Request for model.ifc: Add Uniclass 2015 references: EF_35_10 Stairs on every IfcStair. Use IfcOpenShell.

First a look at what the model holds.

```python
import ifcopenshell

model = ifcopenshell.open("model.ifc")
print(model.schema)
print("classifications:", [c.Name for c in model.by_type("IfcClassification")])
for ifc_class in ("IfcDoor", "IfcRoof", "IfcStair", "IfcWall", "IfcWindow"):
    print(ifc_class, len(model.by_type(ifc_class)))
```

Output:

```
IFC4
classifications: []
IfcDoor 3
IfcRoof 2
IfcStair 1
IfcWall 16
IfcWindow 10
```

```python
import ifcopenshell
import ifcopenshell.api.classification

model = ifcopenshell.open("model.ifc")

system = ifcopenshell.api.classification.add_classification(model, classification="Uniclass 2015")

codes = {
    "IfcStair": ("EF_35_10", "Stairs"),
}
for ifc_class, (code, name) in codes.items():
    products = model.by_type(ifc_class)
    ifcopenshell.api.classification.add_reference(
        model, products=products, classification=system, identification=code, name=name
    )
    print(code, len(products))

model.write("model_rev.ifc")
```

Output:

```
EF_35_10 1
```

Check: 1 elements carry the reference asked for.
